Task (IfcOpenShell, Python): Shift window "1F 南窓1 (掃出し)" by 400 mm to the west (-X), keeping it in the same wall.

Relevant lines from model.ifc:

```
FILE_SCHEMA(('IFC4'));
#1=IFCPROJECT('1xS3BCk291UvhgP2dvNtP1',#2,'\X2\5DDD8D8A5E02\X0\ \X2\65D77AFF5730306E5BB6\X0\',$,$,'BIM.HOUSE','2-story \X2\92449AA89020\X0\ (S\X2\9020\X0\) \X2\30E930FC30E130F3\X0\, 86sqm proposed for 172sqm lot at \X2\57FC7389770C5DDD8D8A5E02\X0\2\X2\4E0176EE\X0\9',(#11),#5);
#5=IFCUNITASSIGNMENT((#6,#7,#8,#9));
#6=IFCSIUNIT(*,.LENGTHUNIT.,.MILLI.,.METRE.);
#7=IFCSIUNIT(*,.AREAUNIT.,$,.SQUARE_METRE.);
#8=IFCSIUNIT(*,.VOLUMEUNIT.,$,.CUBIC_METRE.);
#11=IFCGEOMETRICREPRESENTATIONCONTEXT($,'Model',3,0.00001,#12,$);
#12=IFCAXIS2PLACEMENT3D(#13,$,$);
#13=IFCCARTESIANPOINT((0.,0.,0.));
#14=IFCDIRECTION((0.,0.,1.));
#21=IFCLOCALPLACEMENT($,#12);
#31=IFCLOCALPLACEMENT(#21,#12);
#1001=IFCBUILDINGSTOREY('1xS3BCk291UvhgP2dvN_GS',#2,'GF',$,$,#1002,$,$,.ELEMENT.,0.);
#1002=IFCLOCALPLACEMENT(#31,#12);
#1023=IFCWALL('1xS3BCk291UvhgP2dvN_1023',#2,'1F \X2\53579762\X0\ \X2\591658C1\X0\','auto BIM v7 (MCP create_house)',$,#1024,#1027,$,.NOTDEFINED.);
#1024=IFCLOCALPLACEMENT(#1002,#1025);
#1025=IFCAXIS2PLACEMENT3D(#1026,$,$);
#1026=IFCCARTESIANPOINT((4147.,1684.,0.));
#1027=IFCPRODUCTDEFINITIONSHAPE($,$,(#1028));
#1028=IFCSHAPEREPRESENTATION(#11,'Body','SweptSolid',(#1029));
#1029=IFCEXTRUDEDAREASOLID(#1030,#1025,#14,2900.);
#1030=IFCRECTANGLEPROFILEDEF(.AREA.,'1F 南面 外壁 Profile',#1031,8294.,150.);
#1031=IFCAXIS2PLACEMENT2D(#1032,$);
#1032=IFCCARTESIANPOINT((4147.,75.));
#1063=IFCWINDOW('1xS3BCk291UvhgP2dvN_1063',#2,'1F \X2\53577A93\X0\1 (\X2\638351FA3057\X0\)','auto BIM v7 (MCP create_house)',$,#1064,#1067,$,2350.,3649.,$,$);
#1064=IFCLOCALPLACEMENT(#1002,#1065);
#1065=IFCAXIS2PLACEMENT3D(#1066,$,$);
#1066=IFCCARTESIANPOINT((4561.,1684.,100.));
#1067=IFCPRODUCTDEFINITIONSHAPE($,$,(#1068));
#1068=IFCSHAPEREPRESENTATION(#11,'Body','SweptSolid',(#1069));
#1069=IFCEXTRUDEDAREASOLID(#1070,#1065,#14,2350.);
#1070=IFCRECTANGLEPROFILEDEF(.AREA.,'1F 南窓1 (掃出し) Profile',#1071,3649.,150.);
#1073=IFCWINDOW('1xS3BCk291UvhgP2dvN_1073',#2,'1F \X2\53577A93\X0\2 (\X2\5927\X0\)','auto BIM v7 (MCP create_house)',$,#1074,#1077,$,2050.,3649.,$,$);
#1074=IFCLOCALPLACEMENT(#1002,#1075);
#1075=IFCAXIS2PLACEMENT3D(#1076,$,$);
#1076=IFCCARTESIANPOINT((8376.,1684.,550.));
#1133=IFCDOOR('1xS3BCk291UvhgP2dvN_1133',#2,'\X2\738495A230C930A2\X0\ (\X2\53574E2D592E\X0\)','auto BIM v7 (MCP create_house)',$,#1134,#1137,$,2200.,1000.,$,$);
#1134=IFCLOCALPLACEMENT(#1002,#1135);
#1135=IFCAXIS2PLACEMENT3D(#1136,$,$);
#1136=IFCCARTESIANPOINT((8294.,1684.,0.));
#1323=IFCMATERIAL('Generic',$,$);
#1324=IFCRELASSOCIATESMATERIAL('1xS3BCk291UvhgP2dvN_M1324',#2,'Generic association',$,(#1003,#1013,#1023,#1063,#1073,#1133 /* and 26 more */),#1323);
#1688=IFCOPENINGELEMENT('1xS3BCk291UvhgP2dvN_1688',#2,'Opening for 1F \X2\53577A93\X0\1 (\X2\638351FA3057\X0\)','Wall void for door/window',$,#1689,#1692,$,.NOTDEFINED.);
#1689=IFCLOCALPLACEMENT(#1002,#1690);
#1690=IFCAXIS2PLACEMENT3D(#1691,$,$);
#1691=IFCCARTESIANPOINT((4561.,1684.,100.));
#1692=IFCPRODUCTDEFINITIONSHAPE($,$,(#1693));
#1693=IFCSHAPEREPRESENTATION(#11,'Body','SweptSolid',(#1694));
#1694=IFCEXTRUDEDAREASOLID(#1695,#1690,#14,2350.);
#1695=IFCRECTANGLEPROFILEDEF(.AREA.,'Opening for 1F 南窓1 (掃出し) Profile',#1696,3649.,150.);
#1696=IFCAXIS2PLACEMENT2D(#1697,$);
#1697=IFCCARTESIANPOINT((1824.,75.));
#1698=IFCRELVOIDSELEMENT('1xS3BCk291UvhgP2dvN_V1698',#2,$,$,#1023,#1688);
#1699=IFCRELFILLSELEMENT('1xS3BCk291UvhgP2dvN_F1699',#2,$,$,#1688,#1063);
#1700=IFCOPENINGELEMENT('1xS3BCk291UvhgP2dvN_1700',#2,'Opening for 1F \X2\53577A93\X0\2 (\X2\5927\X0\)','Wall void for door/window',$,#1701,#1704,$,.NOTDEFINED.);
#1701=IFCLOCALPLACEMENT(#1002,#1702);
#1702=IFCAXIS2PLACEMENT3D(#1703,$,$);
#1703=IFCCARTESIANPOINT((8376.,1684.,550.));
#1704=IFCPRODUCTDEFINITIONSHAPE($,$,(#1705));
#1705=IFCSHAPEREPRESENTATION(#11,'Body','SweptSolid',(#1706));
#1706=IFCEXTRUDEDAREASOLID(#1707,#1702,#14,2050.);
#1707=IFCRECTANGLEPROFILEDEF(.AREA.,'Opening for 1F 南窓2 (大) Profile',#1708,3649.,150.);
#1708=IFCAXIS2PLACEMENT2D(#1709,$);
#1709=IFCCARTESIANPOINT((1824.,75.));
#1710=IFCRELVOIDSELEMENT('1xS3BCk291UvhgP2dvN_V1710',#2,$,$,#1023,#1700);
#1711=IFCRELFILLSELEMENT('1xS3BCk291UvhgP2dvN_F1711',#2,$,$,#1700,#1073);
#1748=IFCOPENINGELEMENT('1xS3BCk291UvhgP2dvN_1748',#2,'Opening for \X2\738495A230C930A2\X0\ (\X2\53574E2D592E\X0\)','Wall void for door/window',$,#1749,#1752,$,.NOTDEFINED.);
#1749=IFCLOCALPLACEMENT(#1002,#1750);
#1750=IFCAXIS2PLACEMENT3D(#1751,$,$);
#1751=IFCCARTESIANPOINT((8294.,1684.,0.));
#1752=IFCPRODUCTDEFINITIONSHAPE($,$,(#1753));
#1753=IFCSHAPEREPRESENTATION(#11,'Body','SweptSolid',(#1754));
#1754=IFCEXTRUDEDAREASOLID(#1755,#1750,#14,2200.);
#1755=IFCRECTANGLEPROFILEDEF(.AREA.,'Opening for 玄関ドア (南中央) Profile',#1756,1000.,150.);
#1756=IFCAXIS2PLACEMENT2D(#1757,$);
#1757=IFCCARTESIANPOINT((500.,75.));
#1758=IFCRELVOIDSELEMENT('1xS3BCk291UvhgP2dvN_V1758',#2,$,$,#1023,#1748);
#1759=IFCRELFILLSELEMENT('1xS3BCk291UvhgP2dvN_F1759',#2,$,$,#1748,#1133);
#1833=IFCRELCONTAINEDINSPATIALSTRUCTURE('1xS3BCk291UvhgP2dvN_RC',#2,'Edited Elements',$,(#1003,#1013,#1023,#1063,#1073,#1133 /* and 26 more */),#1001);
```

```python
import ifcopenshell
import ifcopenshell.api.geometry
import ifcopenshell.util.placement

model = ifcopenshell.open("model.ifc")

window = model.by_id(1063)
opening = window.FillsVoids[0].RelatingOpeningElement
wall = opening.VoidsElements[0].RelatingBuildingElement

wall_matrix = ifcopenshell.util.placement.get_local_placement(wall.ObjectPlacement)
shift = wall_matrix[:3, 0] * -400.0
before = ifcopenshell.util.placement.get_local_placement(window.ObjectPlacement)[:3, 3].copy()

# The window is not placed relative to its opening, so move both.
for product in (opening, window):
    matrix = ifcopenshell.util.placement.get_local_placement(product.ObjectPlacement)
    matrix[:3, 3] += shift
    ifcopenshell.api.geometry.edit_object_placement(model, product=product, matrix=matrix, is_si=False)

after = ifcopenshell.util.placement.get_local_placement(window.ObjectPlacement)[:3, 3]
print("window moved by", (after - before).round(3) + 0.0)

model.write("model_rev.ifc")
```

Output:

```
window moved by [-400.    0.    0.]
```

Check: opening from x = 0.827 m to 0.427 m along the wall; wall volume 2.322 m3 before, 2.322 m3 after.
